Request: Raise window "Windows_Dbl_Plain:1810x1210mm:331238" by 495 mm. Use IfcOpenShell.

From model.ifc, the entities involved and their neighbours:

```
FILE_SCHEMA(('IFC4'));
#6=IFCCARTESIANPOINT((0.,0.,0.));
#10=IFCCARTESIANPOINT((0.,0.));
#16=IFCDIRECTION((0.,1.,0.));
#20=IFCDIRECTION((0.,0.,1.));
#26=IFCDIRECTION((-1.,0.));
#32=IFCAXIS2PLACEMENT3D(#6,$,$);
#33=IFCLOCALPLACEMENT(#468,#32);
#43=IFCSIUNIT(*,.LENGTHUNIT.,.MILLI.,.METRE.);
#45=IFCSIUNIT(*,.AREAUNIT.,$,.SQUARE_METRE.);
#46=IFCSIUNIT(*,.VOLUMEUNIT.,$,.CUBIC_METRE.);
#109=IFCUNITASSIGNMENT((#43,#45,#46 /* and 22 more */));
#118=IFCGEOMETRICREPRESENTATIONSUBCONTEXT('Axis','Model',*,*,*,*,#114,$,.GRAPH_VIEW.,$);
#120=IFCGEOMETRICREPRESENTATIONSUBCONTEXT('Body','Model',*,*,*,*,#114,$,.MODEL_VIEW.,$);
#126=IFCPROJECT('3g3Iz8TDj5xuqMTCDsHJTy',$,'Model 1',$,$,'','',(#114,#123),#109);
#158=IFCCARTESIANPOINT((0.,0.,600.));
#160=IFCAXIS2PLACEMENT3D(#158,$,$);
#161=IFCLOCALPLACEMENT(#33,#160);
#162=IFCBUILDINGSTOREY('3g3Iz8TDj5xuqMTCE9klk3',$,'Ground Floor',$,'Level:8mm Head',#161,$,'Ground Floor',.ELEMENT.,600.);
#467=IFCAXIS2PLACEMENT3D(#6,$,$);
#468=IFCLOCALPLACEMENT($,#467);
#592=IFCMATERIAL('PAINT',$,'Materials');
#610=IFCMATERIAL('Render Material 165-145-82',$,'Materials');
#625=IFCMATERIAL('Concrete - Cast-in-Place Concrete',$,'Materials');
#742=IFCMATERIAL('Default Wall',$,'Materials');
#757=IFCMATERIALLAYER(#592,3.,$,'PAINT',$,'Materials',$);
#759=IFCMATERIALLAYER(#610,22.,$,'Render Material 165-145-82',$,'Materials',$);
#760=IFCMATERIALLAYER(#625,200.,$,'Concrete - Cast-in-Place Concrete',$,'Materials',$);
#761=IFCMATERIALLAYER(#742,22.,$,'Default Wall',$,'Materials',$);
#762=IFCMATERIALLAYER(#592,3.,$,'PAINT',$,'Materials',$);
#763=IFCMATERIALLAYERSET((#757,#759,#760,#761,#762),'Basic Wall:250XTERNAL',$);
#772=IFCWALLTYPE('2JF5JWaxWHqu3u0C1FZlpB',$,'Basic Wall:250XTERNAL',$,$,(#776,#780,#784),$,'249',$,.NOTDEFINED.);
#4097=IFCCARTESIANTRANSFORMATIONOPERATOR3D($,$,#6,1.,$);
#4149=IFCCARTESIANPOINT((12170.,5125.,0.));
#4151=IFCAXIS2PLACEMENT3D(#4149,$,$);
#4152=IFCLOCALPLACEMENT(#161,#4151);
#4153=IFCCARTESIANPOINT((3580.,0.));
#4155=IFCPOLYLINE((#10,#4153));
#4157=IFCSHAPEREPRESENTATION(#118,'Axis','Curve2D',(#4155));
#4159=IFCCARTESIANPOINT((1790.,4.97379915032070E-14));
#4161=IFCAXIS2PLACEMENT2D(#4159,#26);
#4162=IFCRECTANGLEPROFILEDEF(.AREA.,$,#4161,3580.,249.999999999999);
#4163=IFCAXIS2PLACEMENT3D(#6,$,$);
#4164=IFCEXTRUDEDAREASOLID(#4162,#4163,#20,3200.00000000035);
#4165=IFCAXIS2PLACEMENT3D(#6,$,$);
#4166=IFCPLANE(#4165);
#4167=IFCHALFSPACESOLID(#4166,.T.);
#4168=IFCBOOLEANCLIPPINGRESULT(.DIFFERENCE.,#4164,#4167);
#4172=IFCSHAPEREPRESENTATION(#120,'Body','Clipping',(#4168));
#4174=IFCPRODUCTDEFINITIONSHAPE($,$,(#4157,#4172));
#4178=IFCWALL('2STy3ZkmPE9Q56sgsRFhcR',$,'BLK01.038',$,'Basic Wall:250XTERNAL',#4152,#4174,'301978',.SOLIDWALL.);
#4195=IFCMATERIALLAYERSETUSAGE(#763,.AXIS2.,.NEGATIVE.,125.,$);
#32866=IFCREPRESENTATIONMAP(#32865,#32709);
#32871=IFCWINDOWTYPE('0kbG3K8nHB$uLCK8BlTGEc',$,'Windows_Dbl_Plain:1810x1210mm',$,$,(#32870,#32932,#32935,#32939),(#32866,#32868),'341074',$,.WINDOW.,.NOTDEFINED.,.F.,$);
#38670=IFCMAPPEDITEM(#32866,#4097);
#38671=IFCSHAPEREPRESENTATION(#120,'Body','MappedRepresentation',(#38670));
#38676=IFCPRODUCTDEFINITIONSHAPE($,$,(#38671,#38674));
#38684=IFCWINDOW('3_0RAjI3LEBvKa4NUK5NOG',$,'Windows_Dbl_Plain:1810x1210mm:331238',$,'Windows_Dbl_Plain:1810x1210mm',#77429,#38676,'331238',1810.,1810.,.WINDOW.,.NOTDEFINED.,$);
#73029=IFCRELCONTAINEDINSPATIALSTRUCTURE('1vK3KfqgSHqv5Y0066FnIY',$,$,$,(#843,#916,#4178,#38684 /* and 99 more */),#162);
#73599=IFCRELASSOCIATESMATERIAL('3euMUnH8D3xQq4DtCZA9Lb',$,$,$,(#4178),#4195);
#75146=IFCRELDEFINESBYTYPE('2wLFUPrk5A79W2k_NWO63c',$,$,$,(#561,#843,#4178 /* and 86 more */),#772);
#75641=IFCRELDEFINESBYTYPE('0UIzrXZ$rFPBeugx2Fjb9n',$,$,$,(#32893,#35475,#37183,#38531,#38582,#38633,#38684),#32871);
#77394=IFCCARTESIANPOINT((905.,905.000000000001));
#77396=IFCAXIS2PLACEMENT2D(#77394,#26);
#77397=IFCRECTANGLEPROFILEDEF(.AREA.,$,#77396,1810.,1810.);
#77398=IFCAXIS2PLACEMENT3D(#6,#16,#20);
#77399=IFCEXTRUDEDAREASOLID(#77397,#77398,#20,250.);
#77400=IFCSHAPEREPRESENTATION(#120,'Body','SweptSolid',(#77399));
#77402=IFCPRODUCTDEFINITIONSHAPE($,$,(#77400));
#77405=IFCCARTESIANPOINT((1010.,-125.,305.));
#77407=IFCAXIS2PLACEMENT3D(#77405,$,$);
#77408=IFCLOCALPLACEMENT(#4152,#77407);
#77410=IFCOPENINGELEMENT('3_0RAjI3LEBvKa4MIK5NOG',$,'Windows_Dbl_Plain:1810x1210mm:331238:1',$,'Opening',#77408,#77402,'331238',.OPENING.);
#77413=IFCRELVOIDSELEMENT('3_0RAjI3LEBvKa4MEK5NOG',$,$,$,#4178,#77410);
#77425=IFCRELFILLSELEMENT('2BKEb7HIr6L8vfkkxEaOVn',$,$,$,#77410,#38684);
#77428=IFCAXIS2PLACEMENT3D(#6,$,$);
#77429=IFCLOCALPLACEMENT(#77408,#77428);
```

```python
import numpy as np
import ifcopenshell
import ifcopenshell.api.geometry
import ifcopenshell.util.placement
import ifcopenshell.util.unit

model = ifcopenshell.open("model.ifc")
unit_scale = ifcopenshell.util.unit.calculate_unit_scale(model)

window = model.by_id(38684)
opening = window.FillsVoids[0].RelatingOpeningElement
dz = 495.0

shift = np.array([0.0, 0.0, dz])
# The window is placed relative to its opening, so it follows when the opening moves.
matrix = ifcopenshell.util.placement.get_local_placement(opening.ObjectPlacement)
matrix[:3, 3] += shift
ifcopenshell.api.geometry.edit_object_placement(
    model, product=opening, matrix=matrix, is_si=False, should_transform_children=True
)

print(f"moved by {dz * unit_scale:+.3f} m")

model.write("model_edited.ifc")
```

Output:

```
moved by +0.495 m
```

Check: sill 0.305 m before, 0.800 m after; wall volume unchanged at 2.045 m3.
